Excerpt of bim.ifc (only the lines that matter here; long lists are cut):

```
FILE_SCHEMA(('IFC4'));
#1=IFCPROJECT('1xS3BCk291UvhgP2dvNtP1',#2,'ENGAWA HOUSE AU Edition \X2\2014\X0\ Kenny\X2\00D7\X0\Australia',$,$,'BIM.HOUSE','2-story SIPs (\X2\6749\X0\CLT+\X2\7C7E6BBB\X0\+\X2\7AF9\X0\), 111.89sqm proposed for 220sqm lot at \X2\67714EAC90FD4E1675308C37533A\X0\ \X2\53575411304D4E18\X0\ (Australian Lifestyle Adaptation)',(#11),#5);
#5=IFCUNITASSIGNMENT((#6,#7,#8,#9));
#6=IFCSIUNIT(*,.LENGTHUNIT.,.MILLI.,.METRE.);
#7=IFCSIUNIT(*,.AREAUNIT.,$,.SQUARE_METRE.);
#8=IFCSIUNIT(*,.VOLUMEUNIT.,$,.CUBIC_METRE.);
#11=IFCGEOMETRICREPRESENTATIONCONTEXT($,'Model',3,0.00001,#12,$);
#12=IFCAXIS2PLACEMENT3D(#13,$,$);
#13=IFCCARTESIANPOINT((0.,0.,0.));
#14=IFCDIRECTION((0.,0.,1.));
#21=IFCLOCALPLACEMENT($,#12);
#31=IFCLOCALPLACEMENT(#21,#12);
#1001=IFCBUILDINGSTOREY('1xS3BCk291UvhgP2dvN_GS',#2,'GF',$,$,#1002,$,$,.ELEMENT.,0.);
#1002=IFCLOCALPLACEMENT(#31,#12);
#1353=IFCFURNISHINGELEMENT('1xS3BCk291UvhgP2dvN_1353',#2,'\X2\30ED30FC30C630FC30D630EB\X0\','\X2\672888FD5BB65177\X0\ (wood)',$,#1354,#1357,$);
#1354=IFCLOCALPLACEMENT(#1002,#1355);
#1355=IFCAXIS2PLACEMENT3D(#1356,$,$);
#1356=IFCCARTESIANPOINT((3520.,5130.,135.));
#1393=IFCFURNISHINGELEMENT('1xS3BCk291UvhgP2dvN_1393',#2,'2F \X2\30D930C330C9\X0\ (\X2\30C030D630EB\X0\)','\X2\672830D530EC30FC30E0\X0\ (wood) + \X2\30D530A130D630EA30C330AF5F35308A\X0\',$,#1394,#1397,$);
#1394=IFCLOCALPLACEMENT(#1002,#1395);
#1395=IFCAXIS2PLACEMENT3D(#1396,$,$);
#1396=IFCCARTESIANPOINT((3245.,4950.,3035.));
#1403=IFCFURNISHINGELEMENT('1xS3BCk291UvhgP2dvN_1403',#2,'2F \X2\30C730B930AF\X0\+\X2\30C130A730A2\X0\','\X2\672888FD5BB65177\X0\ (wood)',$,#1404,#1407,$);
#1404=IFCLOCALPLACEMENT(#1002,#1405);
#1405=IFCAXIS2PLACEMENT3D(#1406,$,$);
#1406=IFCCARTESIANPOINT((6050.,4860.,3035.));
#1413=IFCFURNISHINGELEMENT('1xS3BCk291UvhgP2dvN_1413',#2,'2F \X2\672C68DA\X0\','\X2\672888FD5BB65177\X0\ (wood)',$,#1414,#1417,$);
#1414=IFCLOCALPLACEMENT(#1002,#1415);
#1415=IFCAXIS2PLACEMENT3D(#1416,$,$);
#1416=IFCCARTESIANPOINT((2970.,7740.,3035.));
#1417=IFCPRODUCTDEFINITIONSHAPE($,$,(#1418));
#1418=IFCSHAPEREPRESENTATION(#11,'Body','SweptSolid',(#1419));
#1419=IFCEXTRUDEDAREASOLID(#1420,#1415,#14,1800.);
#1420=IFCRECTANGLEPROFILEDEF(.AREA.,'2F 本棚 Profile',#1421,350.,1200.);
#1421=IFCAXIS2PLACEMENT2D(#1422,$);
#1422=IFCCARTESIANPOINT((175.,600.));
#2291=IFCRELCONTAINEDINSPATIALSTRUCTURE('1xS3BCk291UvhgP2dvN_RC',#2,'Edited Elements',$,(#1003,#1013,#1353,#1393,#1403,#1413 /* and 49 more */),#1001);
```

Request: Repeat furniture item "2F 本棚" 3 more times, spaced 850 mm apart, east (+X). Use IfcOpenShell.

```python
import numpy as np
import ifcopenshell
import ifcopenshell.api.geometry
import ifcopenshell.api.root
import ifcopenshell.util.element
import ifcopenshell.util.placement
import ifcopenshell.util.unit

model = ifcopenshell.open("bim.ifc")
unit_scale = ifcopenshell.util.unit.calculate_unit_scale(model)


def reuse_history(source, copy):
    """copy_class also copies each property set's owner history, people and application; keep the originals."""
    for rel in copy.IsDefinedBy:
        if rel.is_a("IfcRelDefinesByProperties") and (history := rel.RelatingPropertyDefinition.OwnerHistory):
            rel.RelatingPropertyDefinition.OwnerHistory = source.OwnerHistory
            ifcopenshell.util.element.remove_deep2(model, history)


source = model.by_guid("1xS3BCk291UvhgP2dvN_1413")
base = ifcopenshell.util.placement.get_local_placement(source.ObjectPlacement)
step = np.array([1.0, 0.0, 0.0]) * 0.85 / unit_scale

for i in range(1, 4):
    copy = ifcopenshell.api.root.copy_class(model, product=source)
    copy.Representation = ifcopenshell.util.element.copy_deep(
        model, source.Representation, exclude=["IfcGeometricRepresentationContext", "IfcRepresentationMap"]
    )
    reuse_history(source, copy)
    matrix = base.copy()
    matrix[:3, 3] += i * step
    print("added at", matrix[:3, 3].round(3) + 0.0)
    ifcopenshell.api.geometry.edit_object_placement(model, product=copy, matrix=matrix, is_si=False)

model.write("bim_v2.ifc")
```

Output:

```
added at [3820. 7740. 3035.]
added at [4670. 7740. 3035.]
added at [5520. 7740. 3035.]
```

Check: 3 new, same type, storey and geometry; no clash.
